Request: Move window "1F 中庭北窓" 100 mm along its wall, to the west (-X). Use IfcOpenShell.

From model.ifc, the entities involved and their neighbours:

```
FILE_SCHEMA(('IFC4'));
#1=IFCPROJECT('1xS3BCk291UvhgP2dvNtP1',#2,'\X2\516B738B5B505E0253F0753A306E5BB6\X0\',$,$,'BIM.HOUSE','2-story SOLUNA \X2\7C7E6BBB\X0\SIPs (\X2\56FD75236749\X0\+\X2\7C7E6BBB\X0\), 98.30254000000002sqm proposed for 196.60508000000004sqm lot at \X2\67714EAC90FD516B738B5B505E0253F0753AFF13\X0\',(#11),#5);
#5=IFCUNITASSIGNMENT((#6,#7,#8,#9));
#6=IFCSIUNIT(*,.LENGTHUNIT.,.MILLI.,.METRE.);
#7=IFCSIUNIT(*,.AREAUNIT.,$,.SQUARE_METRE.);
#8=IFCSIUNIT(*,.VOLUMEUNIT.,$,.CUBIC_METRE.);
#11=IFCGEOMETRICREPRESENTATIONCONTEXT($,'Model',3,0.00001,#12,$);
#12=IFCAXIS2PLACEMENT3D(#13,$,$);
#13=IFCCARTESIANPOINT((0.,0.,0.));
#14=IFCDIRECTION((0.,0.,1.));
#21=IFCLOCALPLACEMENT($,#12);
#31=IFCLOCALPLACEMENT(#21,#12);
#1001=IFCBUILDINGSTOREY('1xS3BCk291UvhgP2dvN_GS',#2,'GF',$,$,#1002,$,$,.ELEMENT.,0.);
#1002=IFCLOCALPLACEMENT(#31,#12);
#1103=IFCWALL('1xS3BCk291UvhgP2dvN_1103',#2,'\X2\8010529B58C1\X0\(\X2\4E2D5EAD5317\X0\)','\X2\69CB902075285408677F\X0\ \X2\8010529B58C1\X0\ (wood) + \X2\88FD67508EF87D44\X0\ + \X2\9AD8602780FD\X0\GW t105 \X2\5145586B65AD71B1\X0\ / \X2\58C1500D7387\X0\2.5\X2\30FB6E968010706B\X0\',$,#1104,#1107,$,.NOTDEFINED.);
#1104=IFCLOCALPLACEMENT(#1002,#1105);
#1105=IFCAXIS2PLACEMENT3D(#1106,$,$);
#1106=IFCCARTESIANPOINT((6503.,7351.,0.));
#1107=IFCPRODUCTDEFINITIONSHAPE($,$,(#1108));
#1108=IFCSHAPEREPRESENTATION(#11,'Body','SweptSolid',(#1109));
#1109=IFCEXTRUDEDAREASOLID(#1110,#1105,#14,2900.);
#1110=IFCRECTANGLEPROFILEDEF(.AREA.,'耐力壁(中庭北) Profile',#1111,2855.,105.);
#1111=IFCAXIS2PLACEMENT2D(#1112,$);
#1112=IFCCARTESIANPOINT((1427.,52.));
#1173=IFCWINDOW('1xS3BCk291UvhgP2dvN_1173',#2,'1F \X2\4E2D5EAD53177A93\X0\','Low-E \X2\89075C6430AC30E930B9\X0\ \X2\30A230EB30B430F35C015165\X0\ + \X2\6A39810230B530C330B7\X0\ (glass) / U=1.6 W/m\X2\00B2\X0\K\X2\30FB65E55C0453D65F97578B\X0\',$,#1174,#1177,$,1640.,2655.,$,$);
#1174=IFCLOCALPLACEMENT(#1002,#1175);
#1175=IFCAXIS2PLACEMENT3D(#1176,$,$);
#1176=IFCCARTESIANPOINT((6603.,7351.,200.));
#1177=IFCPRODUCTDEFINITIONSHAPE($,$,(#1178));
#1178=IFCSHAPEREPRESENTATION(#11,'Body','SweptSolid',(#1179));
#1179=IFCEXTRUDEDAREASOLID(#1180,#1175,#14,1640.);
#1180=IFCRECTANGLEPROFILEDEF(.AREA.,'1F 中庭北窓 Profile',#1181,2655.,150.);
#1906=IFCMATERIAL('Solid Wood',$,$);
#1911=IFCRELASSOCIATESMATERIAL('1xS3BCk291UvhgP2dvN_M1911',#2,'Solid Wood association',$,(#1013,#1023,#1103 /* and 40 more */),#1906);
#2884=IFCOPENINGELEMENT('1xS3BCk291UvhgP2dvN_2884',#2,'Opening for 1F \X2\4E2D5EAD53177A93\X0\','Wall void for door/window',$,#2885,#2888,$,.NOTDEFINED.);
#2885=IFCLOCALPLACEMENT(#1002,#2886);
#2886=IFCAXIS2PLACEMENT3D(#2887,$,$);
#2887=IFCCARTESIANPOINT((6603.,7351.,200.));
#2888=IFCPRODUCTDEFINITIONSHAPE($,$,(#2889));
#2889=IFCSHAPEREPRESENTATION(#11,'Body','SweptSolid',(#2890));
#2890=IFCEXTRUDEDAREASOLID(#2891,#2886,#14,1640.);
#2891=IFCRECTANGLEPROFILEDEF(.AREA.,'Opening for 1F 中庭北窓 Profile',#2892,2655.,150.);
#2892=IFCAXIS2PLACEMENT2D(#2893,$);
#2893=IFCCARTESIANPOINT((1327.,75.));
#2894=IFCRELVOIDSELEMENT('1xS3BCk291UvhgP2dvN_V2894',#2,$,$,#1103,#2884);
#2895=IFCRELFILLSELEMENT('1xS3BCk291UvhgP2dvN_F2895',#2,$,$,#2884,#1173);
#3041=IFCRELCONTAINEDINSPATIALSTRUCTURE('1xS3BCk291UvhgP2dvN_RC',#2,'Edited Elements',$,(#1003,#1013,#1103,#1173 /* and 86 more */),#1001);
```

```python
import ifcopenshell
import ifcopenshell.api.geometry
import ifcopenshell.util.placement
import ifcopenshell.util.unit

model = ifcopenshell.open("model.ifc")
unit_scale = ifcopenshell.util.unit.calculate_unit_scale(model)

window = model.by_id(1173)
opening = window.FillsVoids[0].RelatingOpeningElement
wall = opening.VoidsElements[0].RelatingBuildingElement

wall_matrix = ifcopenshell.util.placement.get_local_placement(wall.ObjectPlacement)
shift = wall_matrix[:3, 0] * -0.1 / unit_scale
before = ifcopenshell.util.placement.get_local_placement(window.ObjectPlacement)[:3, 3].copy()

# The window is not placed relative to its opening, so move both.
for product in (opening, window):
    matrix = ifcopenshell.util.placement.get_local_placement(product.ObjectPlacement)
    matrix[:3, 3] += shift
    ifcopenshell.api.geometry.edit_object_placement(model, product=product, matrix=matrix, is_si=False)

after = ifcopenshell.util.placement.get_local_placement(window.ObjectPlacement)[:3, 3]
print("window moved by", (after - before).round(3) + 0.0)

model.write("model-out.ifc")
```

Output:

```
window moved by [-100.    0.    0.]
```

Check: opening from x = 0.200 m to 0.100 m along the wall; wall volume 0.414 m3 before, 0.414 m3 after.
